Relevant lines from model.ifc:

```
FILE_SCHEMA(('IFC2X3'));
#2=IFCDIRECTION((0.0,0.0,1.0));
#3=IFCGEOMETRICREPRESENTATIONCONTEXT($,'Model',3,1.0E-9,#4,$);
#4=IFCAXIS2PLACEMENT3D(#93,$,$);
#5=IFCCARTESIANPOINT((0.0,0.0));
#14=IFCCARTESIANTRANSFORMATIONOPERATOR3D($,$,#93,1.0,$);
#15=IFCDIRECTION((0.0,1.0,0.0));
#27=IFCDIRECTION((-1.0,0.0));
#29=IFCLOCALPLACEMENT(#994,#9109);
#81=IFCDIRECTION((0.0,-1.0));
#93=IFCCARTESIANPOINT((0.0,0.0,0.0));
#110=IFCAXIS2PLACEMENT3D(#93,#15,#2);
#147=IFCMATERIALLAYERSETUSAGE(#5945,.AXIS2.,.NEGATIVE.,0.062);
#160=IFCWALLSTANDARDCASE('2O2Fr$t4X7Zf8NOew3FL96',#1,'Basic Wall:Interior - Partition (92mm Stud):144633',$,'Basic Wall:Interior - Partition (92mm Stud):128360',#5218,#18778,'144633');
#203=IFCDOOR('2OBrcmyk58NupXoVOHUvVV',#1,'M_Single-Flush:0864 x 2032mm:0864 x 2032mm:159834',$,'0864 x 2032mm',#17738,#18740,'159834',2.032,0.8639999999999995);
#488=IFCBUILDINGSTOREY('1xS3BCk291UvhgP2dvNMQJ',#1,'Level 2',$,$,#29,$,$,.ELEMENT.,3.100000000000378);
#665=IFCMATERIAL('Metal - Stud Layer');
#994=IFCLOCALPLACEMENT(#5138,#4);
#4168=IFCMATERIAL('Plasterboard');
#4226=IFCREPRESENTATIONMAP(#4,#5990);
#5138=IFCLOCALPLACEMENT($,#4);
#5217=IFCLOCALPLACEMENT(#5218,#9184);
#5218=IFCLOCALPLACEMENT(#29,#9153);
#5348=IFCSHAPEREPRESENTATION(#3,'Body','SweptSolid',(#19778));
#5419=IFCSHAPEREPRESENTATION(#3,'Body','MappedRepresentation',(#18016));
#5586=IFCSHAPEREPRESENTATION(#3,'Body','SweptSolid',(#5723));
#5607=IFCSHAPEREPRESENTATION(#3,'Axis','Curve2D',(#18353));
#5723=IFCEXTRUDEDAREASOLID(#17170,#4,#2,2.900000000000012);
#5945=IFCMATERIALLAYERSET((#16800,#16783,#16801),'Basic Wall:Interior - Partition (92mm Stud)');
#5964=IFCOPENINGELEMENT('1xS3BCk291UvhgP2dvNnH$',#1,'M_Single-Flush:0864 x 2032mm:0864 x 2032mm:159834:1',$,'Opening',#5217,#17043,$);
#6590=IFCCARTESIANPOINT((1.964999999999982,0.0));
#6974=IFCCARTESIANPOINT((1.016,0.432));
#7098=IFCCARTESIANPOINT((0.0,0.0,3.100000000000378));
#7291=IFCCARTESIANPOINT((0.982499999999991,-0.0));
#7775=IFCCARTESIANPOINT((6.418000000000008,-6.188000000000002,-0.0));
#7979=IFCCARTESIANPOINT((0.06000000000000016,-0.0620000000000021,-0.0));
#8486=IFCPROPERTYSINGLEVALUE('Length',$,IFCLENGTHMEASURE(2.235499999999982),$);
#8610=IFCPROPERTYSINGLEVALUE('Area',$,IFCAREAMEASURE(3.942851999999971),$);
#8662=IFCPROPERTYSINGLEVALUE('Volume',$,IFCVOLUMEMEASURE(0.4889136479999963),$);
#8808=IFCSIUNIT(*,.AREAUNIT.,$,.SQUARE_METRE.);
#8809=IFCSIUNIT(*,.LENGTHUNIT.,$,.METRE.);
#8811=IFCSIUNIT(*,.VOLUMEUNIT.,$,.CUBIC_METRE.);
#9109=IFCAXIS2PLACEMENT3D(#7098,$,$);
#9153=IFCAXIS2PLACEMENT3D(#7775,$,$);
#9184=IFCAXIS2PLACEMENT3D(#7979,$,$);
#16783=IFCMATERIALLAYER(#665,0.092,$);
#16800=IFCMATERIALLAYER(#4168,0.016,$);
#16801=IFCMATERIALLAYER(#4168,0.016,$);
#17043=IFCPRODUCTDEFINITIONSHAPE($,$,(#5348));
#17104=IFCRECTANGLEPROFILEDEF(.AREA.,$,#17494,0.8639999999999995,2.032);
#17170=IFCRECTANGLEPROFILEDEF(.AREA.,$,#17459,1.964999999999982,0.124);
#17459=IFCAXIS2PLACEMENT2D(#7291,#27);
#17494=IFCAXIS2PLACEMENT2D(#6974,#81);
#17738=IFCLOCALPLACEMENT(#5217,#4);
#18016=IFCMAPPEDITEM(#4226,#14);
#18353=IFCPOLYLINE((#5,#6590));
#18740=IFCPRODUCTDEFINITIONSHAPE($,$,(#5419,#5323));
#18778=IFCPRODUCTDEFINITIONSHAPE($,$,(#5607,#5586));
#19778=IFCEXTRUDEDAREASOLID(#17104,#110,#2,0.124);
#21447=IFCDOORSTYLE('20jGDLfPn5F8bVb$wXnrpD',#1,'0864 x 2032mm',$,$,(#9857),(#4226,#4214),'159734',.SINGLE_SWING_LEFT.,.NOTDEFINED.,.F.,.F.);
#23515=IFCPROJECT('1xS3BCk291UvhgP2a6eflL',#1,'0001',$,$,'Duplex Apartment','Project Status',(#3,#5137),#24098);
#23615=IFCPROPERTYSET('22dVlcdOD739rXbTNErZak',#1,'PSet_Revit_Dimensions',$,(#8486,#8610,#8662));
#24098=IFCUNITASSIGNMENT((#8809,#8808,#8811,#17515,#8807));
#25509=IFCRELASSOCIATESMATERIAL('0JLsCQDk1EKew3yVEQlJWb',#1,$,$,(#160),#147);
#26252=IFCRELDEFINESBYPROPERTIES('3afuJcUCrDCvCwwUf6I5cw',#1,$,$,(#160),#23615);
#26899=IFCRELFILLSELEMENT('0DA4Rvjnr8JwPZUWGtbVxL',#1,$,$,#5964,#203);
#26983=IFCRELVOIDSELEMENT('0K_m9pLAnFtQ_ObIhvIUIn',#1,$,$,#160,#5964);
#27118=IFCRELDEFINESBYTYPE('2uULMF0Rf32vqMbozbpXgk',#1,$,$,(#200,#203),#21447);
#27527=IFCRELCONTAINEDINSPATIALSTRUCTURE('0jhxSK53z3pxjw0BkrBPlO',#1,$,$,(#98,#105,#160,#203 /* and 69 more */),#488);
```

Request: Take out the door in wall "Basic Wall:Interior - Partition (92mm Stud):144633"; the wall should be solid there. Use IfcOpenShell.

```python
import ifcopenshell
import ifcopenshell.api.feature
import ifcopenshell.api.pset
import ifcopenshell.api.root
import ifcopenshell.geom
import ifcopenshell.util.element
import ifcopenshell.util.shape
import ifcopenshell.util.unit

model = ifcopenshell.open("model.ifc")
area_scale = ifcopenshell.util.unit.calculate_unit_scale(model, "AREAUNIT")
volume_scale = ifcopenshell.util.unit.calculate_unit_scale(model, "VOLUMEUNIT")
settings = ifcopenshell.geom.settings()


def volume(element):
    """Net volume in cubic metres, openings subtracted."""
    shape = ifcopenshell.geom.create_shape(settings, element)
    return ifcopenshell.util.shape.get_volume(shape.geometry)


door = model.by_guid("2OBrcmyk58NupXoVOHUvVV")
opening = door.FillsVoids[0].RelatingOpeningElement
wall = opening.VoidsElements[0].RelatingBuildingElement
before = volume(wall)

ifcopenshell.api.root.remove_product(model, product=door)
ifcopenshell.api.feature.remove_feature(model, feature=opening)

after = volume(wall)
thickness = 0.124  # wall thickness in metres

# Update the wall's stored quantities.
pset = model.by_id(ifcopenshell.util.element.get_pset(wall, "PSet_Revit_Dimensions", should_inherit=False)["id"])
ifcopenshell.api.pset.edit_pset(model, pset=pset, properties={
    "Area": model.create_entity("IfcAreaMeasure", after / thickness / area_scale),
    "Volume": model.create_entity("IfcVolumeMeasure", after / volume_scale),
})

print(f"wall volume {before:.3f} -> {after:.3f} m3")

model.write("model_rev.ifc")
```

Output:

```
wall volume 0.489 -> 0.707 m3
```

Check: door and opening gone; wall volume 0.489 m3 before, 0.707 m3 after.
